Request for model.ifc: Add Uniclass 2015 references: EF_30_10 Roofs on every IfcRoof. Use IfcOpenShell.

First a look at what the model holds.

```python
import ifcopenshell

model = ifcopenshell.open("model.ifc")
print(model.schema)
print("classifications:", [c.Name for c in model.by_type("IfcClassification")])
for ifc_class in ("IfcDoor", "IfcRoof", "IfcStair", "IfcWall", "IfcWindow"):
    print(ifc_class, len(model.by_type(ifc_class)))
```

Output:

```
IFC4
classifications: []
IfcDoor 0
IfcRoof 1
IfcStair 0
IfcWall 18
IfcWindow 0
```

```python
import ifcopenshell
import ifcopenshell.api.classification

model = ifcopenshell.open("model.ifc")

system = ifcopenshell.api.classification.add_classification(model, classification="Uniclass 2015")

codes = {
    "IfcRoof": ("EF_30_10", "Roofs"),
}
for ifc_class, (code, name) in codes.items():
    products = model.by_type(ifc_class)
    ifcopenshell.api.classification.add_reference(
        model, products=products, classification=system, identification=code, name=name
    )
    print(code, len(products))

model.write("model_v2.ifc")
```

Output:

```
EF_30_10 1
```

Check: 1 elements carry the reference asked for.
